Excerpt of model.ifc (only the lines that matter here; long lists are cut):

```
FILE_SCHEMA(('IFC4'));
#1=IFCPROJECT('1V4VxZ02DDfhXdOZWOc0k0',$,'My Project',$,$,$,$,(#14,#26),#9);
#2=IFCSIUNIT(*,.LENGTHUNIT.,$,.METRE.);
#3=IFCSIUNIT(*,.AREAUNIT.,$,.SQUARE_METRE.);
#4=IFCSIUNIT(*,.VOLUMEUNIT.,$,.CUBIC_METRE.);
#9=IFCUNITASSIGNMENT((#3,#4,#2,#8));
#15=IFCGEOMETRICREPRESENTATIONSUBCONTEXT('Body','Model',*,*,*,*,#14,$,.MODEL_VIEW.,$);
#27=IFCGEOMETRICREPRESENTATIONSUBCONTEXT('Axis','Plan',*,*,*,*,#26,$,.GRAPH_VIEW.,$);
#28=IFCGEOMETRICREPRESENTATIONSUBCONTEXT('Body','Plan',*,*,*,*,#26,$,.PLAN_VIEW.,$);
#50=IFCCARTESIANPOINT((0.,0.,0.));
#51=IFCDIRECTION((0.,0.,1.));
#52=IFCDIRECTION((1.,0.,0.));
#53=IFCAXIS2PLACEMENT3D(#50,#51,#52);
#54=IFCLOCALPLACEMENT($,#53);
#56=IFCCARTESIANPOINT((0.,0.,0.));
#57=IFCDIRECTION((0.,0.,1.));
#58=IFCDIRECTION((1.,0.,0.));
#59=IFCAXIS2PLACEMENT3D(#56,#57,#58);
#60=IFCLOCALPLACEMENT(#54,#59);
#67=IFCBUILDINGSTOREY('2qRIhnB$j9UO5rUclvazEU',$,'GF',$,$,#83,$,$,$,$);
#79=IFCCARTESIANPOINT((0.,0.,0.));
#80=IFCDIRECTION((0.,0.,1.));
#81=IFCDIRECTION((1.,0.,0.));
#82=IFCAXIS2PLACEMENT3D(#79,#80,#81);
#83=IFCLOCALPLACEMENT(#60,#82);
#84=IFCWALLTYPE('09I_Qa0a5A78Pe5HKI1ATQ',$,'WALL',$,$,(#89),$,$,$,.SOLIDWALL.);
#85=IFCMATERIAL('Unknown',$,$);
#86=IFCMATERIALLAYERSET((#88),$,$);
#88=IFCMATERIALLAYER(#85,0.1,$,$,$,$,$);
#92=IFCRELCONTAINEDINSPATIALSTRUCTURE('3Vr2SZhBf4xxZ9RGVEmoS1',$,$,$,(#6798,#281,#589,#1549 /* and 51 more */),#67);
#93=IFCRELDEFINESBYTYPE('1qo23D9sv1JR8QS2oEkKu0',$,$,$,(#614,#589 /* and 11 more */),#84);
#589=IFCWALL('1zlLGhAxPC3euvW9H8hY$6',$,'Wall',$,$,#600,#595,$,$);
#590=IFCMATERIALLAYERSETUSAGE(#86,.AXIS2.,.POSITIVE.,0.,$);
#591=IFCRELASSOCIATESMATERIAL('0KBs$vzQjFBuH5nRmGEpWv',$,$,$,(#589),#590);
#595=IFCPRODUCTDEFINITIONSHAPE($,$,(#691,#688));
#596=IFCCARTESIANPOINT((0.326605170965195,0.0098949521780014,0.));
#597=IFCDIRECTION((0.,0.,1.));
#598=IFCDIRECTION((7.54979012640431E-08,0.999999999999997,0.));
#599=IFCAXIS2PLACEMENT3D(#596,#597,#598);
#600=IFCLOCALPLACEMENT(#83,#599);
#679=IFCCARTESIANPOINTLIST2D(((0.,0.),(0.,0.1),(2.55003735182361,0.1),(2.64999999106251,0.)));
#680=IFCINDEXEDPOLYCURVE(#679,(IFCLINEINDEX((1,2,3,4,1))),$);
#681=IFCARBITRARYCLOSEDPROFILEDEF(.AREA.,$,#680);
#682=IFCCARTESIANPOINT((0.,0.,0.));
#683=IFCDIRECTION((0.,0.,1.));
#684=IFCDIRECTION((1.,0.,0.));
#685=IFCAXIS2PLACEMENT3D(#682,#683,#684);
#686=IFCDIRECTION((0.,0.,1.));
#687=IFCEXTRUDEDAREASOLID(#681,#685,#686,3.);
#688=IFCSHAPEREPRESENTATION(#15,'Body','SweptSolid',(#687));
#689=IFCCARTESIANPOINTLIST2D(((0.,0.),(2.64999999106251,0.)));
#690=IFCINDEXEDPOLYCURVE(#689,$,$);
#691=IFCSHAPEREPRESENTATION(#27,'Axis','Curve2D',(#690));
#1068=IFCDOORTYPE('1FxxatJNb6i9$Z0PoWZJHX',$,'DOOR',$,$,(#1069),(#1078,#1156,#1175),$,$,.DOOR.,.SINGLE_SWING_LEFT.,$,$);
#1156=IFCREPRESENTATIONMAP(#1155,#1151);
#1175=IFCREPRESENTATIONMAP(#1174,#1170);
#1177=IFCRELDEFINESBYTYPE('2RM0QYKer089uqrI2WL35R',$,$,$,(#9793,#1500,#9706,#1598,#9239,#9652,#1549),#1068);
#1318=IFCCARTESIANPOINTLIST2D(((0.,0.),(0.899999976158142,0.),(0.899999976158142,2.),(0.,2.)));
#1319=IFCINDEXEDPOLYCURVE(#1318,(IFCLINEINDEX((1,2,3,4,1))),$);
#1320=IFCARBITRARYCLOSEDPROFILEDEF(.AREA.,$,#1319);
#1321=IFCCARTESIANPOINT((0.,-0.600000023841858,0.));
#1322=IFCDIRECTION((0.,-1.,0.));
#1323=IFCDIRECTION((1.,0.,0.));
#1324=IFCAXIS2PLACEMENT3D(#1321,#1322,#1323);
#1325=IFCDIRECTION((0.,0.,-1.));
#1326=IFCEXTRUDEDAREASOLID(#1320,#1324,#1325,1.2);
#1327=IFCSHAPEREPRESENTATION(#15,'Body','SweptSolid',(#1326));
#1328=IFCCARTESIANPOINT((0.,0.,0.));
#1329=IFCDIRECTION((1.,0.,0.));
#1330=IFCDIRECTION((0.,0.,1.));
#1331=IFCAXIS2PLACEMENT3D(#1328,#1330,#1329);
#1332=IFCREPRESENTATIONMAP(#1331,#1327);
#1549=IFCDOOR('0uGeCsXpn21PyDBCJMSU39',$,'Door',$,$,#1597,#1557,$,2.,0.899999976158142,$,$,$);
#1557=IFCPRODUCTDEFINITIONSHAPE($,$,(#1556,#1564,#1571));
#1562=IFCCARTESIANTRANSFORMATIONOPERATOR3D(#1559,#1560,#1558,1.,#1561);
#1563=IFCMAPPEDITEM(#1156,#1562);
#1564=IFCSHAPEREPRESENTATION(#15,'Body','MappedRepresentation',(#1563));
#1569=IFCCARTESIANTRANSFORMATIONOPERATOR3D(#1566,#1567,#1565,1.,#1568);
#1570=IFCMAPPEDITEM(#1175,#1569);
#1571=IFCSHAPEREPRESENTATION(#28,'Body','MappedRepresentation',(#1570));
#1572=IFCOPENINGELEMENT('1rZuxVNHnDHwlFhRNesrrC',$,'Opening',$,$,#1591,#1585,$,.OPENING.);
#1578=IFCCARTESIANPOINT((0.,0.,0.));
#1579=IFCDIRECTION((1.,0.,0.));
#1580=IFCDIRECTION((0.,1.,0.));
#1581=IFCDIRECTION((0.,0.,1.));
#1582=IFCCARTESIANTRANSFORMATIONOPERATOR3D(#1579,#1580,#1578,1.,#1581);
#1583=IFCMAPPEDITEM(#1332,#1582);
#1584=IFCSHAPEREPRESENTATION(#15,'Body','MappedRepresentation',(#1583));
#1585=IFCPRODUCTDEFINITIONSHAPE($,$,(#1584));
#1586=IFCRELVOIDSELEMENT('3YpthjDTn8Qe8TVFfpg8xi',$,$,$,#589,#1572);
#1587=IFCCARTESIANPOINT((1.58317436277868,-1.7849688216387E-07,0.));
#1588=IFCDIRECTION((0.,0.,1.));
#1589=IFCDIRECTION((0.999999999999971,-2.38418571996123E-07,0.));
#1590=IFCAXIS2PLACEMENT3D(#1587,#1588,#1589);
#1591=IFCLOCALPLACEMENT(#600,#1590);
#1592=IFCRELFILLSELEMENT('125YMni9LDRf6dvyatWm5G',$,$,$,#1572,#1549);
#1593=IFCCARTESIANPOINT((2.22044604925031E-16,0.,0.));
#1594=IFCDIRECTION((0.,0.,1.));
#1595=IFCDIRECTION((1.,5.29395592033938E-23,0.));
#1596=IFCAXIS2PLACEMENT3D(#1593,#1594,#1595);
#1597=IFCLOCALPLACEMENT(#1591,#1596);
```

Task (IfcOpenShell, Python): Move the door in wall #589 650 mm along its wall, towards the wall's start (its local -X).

```python
import ifcopenshell
import ifcopenshell.api.geometry
import ifcopenshell.util.placement
import ifcopenshell.util.unit

model = ifcopenshell.open("model.ifc")
unit_scale = ifcopenshell.util.unit.calculate_unit_scale(model)

door = model.by_id(1549)
opening = door.FillsVoids[0].RelatingOpeningElement
wall = opening.VoidsElements[0].RelatingBuildingElement

wall_matrix = ifcopenshell.util.placement.get_local_placement(wall.ObjectPlacement)
shift = wall_matrix[:3, 0] * -0.65 / unit_scale
before = ifcopenshell.util.placement.get_local_placement(door.ObjectPlacement)[:3, 3].copy()

# The door is placed relative to its opening, so it follows when the opening moves.
matrix = ifcopenshell.util.placement.get_local_placement(opening.ObjectPlacement)
matrix[:3, 3] += shift
ifcopenshell.api.geometry.edit_object_placement(
    model, product=opening, matrix=matrix, is_si=False, should_transform_children=True
)

after = ifcopenshell.util.placement.get_local_placement(door.ObjectPlacement)[:3, 3]
print("door moved by", (after - before).round(3) + 0.0)

model.write("model_edited.ifc")
```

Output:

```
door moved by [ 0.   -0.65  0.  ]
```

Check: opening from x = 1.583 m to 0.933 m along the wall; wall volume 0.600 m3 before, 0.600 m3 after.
